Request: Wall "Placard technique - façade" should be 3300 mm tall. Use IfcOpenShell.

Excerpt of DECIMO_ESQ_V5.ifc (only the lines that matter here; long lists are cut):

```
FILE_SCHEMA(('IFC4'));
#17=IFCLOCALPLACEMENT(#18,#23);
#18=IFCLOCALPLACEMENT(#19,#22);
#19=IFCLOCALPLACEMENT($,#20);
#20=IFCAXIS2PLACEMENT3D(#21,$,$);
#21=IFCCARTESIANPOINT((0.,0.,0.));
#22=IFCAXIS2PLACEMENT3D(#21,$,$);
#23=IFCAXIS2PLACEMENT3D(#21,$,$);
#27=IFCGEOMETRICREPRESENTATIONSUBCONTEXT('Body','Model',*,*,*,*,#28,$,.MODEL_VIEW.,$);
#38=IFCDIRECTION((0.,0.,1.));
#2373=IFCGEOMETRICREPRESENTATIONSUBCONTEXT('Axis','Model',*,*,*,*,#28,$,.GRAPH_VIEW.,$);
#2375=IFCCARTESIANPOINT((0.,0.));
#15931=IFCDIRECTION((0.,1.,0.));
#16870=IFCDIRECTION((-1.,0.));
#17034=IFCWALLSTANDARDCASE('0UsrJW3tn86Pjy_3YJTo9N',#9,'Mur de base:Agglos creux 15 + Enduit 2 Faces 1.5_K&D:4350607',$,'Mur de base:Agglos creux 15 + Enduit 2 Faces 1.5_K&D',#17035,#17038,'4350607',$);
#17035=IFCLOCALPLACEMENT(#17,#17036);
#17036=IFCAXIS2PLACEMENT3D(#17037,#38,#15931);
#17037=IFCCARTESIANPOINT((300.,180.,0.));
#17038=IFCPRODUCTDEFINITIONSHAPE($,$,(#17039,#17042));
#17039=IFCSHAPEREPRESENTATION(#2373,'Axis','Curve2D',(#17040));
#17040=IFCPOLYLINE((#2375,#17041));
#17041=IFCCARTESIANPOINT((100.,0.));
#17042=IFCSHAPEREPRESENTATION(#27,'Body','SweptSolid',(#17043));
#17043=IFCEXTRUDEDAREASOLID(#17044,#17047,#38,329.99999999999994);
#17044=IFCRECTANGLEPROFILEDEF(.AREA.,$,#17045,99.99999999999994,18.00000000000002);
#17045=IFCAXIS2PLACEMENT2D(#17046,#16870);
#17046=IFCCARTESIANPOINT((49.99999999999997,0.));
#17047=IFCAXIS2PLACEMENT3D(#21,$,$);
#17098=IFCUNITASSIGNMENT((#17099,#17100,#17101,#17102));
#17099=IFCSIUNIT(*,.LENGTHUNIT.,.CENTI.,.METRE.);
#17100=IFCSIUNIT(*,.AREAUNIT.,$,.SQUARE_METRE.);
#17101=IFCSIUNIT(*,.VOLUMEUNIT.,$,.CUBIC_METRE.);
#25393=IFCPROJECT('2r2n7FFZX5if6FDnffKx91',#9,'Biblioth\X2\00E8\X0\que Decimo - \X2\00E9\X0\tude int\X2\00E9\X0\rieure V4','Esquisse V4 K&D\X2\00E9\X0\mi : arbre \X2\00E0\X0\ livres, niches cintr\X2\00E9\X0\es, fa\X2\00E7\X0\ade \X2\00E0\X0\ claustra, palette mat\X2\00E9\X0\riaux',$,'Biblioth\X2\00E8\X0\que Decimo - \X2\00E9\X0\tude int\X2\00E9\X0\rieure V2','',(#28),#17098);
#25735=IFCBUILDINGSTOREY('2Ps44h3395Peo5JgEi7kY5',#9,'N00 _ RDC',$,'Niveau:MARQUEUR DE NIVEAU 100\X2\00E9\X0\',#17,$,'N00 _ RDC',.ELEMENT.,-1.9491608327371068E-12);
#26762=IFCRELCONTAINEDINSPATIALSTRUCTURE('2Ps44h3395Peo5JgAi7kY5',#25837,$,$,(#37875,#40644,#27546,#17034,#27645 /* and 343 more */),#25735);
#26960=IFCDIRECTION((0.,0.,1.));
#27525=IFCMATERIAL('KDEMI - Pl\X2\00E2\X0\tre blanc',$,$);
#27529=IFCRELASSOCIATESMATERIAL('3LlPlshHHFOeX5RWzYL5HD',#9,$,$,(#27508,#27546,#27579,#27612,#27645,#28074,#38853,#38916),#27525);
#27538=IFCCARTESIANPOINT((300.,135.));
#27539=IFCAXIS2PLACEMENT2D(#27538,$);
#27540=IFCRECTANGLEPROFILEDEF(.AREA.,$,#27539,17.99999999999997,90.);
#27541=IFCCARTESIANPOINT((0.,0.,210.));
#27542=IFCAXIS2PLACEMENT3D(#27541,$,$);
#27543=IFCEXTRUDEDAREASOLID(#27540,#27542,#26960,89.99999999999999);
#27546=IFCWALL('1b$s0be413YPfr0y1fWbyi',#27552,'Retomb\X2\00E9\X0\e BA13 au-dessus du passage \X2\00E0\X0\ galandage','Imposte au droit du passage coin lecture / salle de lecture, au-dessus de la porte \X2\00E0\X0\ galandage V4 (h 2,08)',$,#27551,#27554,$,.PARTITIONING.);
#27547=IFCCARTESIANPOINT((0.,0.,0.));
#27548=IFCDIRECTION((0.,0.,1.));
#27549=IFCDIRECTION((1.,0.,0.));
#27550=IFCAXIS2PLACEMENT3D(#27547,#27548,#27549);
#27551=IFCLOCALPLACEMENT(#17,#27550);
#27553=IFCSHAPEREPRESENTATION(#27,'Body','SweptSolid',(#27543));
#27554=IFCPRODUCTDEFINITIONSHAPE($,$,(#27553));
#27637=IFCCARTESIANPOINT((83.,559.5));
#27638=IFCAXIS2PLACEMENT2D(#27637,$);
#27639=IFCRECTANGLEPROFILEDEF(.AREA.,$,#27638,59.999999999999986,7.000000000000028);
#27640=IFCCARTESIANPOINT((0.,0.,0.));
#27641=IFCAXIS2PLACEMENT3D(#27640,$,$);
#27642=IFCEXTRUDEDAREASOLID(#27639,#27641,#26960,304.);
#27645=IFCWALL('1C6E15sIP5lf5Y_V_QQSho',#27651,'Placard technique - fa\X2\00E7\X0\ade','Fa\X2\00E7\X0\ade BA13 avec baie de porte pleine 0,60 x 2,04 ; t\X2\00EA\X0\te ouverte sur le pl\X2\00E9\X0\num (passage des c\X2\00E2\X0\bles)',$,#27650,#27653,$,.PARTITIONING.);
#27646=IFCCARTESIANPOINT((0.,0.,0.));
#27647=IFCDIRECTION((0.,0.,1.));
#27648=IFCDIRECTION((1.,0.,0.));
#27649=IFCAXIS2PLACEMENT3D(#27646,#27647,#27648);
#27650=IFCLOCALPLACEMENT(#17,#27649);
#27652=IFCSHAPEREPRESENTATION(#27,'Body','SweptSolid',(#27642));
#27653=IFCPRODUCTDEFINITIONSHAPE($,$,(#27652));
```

```python
import ifcopenshell
import ifcopenshell.geom
import ifcopenshell.util.representation
import ifcopenshell.util.shape
import ifcopenshell.util.unit

model = ifcopenshell.open("DECIMO_ESQ_V5.ifc")
unit_scale = ifcopenshell.util.unit.calculate_unit_scale(model)
settings = ifcopenshell.geom.settings()


def volume(element):
    """Net volume in cubic metres, openings subtracted."""
    shape = ifcopenshell.geom.create_shape(settings, element)
    return ifcopenshell.util.shape.get_volume(shape.geometry)


wall = model.by_guid("1C6E15sIP5lf5Y_V_QQSho")
before = volume(wall)

body = ifcopenshell.util.representation.get_representation(wall, "Model", "Body")
solid = body.Items[0]
old_height = solid.Depth
solid.Depth = 3.3 / unit_scale
after = volume(wall)

print(f"height {old_height:g} -> {solid.Depth:g}, volume {before:.3f} -> {after:.3f} m3")

model.write("DECIMO_ESQ_V5-out.ifc")
```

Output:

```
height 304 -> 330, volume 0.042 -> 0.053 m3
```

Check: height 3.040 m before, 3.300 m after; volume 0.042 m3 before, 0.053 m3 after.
